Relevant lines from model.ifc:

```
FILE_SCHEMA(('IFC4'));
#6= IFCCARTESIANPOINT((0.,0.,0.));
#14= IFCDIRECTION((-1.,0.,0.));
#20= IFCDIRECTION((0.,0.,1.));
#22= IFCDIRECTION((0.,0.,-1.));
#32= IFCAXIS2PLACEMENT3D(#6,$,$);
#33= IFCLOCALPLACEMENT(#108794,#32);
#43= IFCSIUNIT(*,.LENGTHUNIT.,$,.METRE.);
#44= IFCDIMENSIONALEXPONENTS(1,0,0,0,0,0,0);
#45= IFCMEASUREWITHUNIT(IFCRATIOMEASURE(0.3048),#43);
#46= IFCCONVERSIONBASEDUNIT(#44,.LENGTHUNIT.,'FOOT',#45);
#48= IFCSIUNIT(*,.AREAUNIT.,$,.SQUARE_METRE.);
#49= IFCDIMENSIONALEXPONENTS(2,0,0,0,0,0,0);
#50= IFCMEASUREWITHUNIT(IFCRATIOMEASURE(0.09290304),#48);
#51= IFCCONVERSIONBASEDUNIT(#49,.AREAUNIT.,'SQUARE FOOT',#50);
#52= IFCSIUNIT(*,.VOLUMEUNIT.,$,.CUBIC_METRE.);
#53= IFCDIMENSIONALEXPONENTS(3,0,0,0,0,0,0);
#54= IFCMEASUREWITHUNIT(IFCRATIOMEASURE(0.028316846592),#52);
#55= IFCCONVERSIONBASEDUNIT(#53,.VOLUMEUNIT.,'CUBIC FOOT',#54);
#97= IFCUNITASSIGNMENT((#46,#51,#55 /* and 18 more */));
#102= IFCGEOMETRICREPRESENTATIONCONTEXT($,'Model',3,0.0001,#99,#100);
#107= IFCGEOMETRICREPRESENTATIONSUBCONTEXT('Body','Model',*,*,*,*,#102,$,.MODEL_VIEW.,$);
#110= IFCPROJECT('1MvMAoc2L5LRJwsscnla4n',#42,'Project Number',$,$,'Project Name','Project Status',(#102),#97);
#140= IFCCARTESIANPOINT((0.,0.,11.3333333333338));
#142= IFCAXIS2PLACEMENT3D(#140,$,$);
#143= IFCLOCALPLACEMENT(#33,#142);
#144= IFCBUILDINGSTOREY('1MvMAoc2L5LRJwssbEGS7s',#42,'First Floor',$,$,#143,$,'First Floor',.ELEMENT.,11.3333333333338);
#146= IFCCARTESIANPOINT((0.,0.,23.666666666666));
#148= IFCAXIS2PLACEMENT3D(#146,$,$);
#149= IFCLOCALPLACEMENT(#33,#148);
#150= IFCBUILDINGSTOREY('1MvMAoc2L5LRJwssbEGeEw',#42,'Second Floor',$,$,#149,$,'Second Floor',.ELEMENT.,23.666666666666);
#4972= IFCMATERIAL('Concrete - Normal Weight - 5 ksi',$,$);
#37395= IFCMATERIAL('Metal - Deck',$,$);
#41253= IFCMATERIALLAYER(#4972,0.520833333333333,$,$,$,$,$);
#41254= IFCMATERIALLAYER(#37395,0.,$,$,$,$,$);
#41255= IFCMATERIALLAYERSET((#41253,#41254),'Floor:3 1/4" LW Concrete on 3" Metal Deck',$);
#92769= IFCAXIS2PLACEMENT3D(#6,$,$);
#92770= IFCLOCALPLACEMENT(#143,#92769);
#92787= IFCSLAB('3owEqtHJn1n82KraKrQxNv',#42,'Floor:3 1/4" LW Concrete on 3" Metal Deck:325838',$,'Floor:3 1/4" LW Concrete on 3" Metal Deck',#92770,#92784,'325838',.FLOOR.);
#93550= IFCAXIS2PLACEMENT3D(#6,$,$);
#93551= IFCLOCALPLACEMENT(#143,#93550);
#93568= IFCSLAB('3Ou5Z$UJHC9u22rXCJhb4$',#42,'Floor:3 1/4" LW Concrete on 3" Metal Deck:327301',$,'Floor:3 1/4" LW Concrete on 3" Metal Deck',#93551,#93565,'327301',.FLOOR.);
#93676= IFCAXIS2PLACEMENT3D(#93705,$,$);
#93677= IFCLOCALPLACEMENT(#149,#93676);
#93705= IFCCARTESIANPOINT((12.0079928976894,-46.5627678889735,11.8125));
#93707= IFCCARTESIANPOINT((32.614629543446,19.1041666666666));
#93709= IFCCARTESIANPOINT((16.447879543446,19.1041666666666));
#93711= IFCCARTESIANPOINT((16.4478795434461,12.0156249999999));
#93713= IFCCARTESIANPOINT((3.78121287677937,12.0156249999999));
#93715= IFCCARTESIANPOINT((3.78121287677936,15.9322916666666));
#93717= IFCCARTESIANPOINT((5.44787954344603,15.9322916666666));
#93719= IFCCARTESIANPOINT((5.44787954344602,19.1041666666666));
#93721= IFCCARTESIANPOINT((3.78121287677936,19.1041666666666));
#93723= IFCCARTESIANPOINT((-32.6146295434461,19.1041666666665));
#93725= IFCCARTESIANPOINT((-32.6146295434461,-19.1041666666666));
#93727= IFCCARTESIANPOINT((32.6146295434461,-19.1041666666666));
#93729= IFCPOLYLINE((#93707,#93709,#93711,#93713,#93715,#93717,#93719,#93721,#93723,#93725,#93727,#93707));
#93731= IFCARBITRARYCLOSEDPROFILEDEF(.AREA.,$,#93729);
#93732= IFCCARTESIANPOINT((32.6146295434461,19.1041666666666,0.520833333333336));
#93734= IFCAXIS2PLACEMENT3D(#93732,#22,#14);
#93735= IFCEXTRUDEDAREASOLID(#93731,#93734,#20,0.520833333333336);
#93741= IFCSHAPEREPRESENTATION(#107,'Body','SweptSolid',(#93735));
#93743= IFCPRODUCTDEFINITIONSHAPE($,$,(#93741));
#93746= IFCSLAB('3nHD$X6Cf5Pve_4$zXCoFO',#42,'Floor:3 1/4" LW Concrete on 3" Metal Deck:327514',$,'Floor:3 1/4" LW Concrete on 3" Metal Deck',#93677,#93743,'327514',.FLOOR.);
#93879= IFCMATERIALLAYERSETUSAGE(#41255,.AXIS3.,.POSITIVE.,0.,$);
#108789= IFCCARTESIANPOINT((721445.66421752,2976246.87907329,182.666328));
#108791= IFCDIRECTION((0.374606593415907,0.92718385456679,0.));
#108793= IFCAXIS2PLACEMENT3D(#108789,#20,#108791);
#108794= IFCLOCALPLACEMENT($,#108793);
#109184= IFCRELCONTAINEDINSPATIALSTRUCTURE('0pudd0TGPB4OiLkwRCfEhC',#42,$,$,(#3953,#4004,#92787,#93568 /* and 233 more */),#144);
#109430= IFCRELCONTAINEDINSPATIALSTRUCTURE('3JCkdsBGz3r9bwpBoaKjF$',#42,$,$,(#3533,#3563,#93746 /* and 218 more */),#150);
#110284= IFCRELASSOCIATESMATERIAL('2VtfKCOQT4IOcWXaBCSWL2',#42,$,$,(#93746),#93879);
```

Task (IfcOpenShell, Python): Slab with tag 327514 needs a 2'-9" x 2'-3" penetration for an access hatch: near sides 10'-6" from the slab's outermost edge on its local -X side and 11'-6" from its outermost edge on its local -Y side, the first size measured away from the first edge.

```python
import numpy as np
import ifcopenshell
import ifcopenshell.api.feature
import ifcopenshell.api.geometry
import ifcopenshell.api.root
import ifcopenshell.geom
import ifcopenshell.util.placement
import ifcopenshell.util.representation
import ifcopenshell.util.shape
import ifcopenshell.util.unit

model = ifcopenshell.open("model.ifc")
unit_scale = ifcopenshell.util.unit.calculate_unit_scale(model)
settings = ifcopenshell.geom.settings()


def volume(element):
    """Net volume in cubic metres, openings subtracted."""
    shape = ifcopenshell.geom.create_shape(settings, element)
    return ifcopenshell.util.shape.get_volume(shape.geometry)


slab = model.by_guid("3nHD$X6Cf5Pve_4$zXCoFO")
before = volume(slab)

# Extent in the slab's own axes, in metres. The edges named are its -X and -Y sides.
slab_shape = ifcopenshell.geom.create_shape(settings, slab)
vertices = ifcopenshell.util.shape.get_vertices(slab_shape.geometry)
x_min, y_min, bottom = vertices.min(axis=0)
top = vertices[:, 2].max()

opening = ifcopenshell.api.root.create_entity(model, ifc_class="IfcOpeningElement", name="Access hatch opening", predefined_type="OPENING")
context = ifcopenshell.util.representation.get_context(model, "Model", "Body", "MODEL_VIEW")
width, depth = 0.8382, 0.6858
outline = [(0.0, 0.0), (width, 0.0), (width, depth), (0.0, depth), (0.0, 0.0)]
# Overshoot both faces by 50 mm so the cut is clean.
shape = ifcopenshell.api.geometry.add_slab_representation(
    model, context=context, depth=top - bottom + 0.1, polyline=outline
)
ifcopenshell.api.geometry.assign_representation(model, product=opening, representation=shape)

matrix = ifcopenshell.util.placement.get_local_placement(slab.ObjectPlacement)
matrix[:, 3] = matrix @ np.append(np.array([x_min + 3.2004, y_min + 3.5052, bottom - 0.05]) / unit_scale, 1.0)
ifcopenshell.api.geometry.edit_object_placement(model, product=opening, matrix=matrix, is_si=False)
ifcopenshell.api.feature.add_feature(model, feature=opening, element=slab)

after = volume(slab)

print(f"slab volume {before:.3f} -> {after:.3f} m3")

model.write("model_v2.ifc")
```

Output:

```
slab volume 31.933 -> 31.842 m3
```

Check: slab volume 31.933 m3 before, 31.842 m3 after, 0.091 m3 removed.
